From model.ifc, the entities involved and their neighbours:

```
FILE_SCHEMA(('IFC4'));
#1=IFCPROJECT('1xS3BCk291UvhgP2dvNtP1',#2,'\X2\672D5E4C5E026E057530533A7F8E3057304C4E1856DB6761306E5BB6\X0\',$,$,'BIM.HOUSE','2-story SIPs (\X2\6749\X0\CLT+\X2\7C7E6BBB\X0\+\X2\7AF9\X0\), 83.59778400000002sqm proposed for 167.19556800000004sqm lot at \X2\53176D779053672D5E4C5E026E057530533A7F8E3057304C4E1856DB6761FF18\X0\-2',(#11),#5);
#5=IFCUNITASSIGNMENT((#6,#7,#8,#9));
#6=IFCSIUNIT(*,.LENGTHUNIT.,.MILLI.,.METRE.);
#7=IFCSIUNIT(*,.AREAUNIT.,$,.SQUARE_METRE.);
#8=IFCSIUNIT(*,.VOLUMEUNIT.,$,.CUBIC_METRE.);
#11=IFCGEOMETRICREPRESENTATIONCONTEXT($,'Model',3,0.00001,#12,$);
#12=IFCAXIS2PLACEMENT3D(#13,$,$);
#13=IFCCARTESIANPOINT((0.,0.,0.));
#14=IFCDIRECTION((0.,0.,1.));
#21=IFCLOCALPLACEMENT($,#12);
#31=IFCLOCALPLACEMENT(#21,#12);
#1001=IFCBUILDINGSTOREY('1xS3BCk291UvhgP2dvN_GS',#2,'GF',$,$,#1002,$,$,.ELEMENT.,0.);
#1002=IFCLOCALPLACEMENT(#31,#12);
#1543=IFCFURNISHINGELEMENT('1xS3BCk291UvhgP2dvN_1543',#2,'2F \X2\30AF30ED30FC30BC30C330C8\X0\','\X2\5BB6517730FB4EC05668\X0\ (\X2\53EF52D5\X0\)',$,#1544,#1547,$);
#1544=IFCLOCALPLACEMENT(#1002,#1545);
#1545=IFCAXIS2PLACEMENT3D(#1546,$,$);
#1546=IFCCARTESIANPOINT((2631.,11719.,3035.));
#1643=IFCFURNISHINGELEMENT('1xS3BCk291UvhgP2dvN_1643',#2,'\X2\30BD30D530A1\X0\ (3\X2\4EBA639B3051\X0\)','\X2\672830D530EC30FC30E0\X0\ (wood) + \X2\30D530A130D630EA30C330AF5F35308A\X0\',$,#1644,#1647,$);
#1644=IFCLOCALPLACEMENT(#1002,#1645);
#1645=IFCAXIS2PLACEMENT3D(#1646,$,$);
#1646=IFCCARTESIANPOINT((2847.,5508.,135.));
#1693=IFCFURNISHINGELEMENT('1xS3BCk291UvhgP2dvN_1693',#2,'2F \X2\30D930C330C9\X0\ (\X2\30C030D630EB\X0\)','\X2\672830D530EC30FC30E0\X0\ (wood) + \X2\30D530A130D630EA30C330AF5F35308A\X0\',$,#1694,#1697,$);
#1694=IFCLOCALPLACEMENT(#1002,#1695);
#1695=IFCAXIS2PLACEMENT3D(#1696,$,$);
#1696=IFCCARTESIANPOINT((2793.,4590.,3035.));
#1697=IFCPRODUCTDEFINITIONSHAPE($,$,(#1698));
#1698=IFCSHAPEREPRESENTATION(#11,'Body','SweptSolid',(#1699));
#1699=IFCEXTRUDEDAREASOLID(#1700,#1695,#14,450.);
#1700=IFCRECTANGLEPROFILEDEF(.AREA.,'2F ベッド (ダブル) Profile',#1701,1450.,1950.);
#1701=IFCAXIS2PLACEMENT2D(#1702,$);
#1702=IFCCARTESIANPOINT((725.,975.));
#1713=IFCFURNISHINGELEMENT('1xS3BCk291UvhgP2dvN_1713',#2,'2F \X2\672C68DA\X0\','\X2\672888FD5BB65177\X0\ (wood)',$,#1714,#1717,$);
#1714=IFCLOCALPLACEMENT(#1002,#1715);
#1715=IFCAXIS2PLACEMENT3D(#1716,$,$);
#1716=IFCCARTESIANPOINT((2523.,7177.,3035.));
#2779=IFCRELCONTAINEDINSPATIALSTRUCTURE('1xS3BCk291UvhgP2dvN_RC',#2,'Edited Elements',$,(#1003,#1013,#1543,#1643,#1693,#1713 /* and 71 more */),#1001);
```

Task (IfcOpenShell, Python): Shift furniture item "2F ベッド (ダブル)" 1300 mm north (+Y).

```python
import ifcopenshell
import ifcopenshell.api.geometry
import ifcopenshell.util.placement
import ifcopenshell.util.unit

model = ifcopenshell.open("model.ifc")
unit_scale = ifcopenshell.util.unit.calculate_unit_scale(model)

item = model.by_id(1693)
matrix = ifcopenshell.util.placement.get_local_placement(item.ObjectPlacement)
matrix[1, 3] += 1.3 / unit_scale
ifcopenshell.api.geometry.edit_object_placement(model, product=item, matrix=matrix, is_si=False)

print(ifcopenshell.util.placement.get_local_placement(item.ObjectPlacement).round(3) + 0.0)

model.write("model_v2.ifc")
```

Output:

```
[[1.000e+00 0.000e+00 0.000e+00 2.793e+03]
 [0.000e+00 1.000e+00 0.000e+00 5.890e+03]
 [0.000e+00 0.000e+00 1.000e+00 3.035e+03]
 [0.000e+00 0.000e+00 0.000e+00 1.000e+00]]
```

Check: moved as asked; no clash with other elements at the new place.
